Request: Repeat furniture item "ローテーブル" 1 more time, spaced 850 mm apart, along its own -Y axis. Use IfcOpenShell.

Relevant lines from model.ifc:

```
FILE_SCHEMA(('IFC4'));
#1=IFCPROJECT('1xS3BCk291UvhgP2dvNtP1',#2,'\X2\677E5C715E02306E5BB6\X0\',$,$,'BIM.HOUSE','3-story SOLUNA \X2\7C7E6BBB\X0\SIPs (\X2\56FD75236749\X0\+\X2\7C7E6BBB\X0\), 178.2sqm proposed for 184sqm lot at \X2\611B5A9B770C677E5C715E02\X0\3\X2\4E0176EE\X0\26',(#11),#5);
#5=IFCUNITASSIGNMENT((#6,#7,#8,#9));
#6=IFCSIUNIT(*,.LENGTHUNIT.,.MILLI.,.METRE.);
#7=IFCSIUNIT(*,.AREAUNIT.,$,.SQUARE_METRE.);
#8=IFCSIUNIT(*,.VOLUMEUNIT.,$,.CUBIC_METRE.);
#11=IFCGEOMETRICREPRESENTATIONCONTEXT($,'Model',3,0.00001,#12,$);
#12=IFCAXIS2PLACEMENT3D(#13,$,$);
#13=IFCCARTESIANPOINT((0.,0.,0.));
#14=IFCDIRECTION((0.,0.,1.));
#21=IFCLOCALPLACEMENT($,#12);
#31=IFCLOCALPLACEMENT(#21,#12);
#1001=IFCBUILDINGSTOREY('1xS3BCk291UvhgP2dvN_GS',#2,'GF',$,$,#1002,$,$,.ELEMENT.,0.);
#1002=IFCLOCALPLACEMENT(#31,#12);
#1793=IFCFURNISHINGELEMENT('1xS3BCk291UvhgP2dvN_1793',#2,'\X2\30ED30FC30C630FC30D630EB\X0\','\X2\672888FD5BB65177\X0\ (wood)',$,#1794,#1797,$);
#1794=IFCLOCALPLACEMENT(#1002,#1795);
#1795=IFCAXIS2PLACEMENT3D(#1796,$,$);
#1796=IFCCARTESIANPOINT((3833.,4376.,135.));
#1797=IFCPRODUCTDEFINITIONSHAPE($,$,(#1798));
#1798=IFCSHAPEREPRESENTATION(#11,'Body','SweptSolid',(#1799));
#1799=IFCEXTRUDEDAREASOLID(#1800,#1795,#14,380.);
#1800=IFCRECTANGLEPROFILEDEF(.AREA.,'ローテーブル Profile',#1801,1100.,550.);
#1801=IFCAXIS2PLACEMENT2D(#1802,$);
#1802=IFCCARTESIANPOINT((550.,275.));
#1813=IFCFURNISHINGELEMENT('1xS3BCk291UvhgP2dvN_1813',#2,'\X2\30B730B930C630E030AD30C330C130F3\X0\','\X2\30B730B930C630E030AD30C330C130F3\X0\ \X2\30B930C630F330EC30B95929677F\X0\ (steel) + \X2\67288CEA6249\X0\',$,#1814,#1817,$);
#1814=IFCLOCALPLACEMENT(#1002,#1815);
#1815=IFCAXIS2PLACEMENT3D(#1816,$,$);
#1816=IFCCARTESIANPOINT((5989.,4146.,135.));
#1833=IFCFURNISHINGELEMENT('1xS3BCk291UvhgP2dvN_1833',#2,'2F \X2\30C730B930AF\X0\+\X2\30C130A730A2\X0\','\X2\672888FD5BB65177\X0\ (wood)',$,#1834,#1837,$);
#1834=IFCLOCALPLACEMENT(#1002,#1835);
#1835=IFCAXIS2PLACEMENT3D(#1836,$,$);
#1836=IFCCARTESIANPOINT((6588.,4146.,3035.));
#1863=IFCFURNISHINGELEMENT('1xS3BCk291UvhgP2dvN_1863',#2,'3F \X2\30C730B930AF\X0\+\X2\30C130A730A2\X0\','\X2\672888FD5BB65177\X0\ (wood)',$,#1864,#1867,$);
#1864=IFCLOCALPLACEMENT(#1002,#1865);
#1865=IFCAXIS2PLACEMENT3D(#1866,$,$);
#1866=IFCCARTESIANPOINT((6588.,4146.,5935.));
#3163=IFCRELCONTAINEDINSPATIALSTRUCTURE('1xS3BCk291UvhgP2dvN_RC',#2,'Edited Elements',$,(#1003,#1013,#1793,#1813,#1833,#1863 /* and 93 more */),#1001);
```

```python
import ifcopenshell
import ifcopenshell.api.geometry
import ifcopenshell.api.root
import ifcopenshell.util.element
import ifcopenshell.util.placement
import ifcopenshell.util.unit

model = ifcopenshell.open("model.ifc")
unit_scale = ifcopenshell.util.unit.calculate_unit_scale(model)


def reuse_history(source, copy):
    """copy_class also copies each property set's owner history, people and application; keep the originals."""
    for rel in copy.IsDefinedBy:
        if rel.is_a("IfcRelDefinesByProperties") and (history := rel.RelatingPropertyDefinition.OwnerHistory):
            rel.RelatingPropertyDefinition.OwnerHistory = source.OwnerHistory
            ifcopenshell.util.element.remove_deep2(model, history)


source = model.by_guid("1xS3BCk291UvhgP2dvN_1793")
base = ifcopenshell.util.placement.get_local_placement(source.ObjectPlacement)
step = -base[:3, 1] * 0.85 / unit_scale

for i in range(1, 2):
    copy = ifcopenshell.api.root.copy_class(model, product=source)
    copy.Representation = ifcopenshell.util.element.copy_deep(
        model, source.Representation, exclude=["IfcGeometricRepresentationContext", "IfcRepresentationMap"]
    )
    reuse_history(source, copy)
    matrix = base.copy()
    matrix[:3, 3] += i * step
    print("added at", matrix[:3, 3].round(3) + 0.0)
    ifcopenshell.api.geometry.edit_object_placement(model, product=copy, matrix=matrix, is_si=False)

model.write("model_v2.ifc")
```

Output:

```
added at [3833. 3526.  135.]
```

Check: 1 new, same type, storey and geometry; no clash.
